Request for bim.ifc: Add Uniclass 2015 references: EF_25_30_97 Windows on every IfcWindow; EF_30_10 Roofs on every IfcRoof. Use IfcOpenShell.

First a look at what the model holds.

```python
import ifcopenshell

model = ifcopenshell.open("bim.ifc")
print(model.schema)
print("classifications:", [c.Name for c in model.by_type("IfcClassification")])
for ifc_class in ("IfcDoor", "IfcRoof", "IfcStair", "IfcWall", "IfcWindow"):
    print(ifc_class, len(model.by_type(ifc_class)))
```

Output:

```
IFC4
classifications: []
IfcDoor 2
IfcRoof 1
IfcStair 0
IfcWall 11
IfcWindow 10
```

```python
import ifcopenshell
import ifcopenshell.api.classification

model = ifcopenshell.open("bim.ifc")

system = ifcopenshell.api.classification.add_classification(model, classification="Uniclass 2015")

codes = {
    "IfcWindow": ("EF_25_30_97", "Windows"),
    "IfcRoof": ("EF_30_10", "Roofs"),
}
for ifc_class, (code, name) in codes.items():
    products = model.by_type(ifc_class)
    ifcopenshell.api.classification.add_reference(
        model, products=products, classification=system, identification=code, name=name
    )
    print(code, len(products))

model.write("bim_edited.ifc")
```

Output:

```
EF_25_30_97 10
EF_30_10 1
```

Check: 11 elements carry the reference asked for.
